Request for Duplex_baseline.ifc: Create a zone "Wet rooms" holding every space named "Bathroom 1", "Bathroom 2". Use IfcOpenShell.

First a look at what the model holds.

```python
import ifcopenshell

model = ifcopenshell.open("Duplex_baseline.ifc")
print(model.schema)
seen = {}
for space in model.by_type("IfcSpace"):
    seen[space.LongName] = seen.get(space.LongName, 0) + 1
for name, count in sorted(seen.items(), key=str):
    print(count, "x", name)
print("zones:", [z.Name for z in model.by_type("IfcZone")][:20])
```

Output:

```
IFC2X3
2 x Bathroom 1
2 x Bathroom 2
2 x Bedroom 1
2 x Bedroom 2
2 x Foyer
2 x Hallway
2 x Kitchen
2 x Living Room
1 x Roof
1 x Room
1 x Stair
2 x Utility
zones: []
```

```python
import ifcopenshell
import ifcopenshell.api.group
import ifcopenshell.api.root

model = ifcopenshell.open("Duplex_baseline.ifc")

names = {"Bathroom 1", "Bathroom 2"}
spaces = [s for s in model.by_type("IfcSpace") if s.LongName in names]

zone = ifcopenshell.api.root.create_entity(model, ifc_class="IfcZone", name="Wet rooms")
ifcopenshell.api.group.assign_group(model, products=spaces, group=zone)
print(len(spaces), "spaces in", zone.Name)

model.write("Duplex_baseline_updated.ifc")
```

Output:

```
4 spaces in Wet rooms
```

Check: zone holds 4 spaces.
